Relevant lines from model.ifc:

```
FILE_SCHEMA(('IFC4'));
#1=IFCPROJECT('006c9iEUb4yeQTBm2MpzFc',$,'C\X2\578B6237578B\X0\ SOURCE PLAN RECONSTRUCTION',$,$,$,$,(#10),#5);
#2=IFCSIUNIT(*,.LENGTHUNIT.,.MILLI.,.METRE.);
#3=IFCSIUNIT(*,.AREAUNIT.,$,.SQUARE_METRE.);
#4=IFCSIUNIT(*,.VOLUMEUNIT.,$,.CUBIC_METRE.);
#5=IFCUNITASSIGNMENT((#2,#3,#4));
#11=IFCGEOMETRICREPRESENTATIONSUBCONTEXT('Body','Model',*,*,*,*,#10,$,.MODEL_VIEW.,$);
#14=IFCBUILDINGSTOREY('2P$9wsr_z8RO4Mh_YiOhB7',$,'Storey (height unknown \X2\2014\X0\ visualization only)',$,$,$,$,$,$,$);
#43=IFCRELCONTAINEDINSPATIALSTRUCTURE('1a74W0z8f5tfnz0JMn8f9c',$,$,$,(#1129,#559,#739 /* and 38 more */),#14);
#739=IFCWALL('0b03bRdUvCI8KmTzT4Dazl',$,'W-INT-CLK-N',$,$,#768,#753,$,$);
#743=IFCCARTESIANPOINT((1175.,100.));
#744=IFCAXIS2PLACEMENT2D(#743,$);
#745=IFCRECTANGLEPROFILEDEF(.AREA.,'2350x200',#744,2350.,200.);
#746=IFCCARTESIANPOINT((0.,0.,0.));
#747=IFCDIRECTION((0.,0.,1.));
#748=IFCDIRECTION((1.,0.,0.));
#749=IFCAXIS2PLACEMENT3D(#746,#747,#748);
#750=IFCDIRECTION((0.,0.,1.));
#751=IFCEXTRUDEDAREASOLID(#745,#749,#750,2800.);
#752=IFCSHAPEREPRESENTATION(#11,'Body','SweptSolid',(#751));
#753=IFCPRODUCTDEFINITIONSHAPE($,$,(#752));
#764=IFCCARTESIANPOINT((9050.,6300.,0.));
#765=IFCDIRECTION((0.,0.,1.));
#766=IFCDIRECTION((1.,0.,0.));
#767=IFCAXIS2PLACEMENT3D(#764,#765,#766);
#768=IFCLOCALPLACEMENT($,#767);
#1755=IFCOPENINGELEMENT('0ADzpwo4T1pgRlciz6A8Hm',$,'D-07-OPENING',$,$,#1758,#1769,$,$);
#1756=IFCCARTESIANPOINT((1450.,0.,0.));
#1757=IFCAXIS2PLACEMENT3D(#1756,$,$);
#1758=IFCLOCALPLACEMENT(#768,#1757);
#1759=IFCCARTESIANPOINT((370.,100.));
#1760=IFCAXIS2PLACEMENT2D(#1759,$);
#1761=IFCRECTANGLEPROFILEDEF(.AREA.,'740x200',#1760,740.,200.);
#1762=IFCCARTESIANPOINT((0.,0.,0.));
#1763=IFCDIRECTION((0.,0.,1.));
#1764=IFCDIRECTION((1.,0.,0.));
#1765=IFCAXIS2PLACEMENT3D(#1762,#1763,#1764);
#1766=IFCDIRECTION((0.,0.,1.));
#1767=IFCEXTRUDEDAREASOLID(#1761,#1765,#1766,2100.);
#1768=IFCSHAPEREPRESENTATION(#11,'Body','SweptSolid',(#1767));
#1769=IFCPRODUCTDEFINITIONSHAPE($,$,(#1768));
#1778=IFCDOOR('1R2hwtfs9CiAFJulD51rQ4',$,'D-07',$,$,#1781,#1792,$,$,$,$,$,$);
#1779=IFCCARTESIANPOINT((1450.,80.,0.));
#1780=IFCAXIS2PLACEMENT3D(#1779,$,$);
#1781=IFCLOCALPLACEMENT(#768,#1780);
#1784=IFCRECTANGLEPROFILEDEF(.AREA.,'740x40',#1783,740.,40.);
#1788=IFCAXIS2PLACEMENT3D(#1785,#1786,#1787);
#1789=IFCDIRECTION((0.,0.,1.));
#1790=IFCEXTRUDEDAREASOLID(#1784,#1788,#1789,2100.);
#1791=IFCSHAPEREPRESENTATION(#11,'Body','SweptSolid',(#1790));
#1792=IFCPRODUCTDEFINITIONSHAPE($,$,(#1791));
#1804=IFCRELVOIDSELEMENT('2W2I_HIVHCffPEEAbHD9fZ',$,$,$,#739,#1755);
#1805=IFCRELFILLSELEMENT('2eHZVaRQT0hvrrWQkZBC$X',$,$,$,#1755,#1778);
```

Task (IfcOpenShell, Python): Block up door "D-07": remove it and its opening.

```python
import ifcopenshell
import ifcopenshell.api.feature
import ifcopenshell.api.root
import ifcopenshell.geom
import ifcopenshell.util.shape

model = ifcopenshell.open("model.ifc")
settings = ifcopenshell.geom.settings()


def volume(element):
    """Net volume in cubic metres, openings subtracted."""
    shape = ifcopenshell.geom.create_shape(settings, element)
    return ifcopenshell.util.shape.get_volume(shape.geometry)


door = model.by_id(1778)
opening = door.FillsVoids[0].RelatingOpeningElement
wall = opening.VoidsElements[0].RelatingBuildingElement
before = volume(wall)

ifcopenshell.api.root.remove_product(model, product=door)
ifcopenshell.api.feature.remove_feature(model, feature=opening)

after = volume(wall)

print(f"wall volume {before:.3f} -> {after:.3f} m3")

model.write("model_updated.ifc")
```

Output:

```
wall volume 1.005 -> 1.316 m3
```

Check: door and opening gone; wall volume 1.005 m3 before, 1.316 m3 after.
